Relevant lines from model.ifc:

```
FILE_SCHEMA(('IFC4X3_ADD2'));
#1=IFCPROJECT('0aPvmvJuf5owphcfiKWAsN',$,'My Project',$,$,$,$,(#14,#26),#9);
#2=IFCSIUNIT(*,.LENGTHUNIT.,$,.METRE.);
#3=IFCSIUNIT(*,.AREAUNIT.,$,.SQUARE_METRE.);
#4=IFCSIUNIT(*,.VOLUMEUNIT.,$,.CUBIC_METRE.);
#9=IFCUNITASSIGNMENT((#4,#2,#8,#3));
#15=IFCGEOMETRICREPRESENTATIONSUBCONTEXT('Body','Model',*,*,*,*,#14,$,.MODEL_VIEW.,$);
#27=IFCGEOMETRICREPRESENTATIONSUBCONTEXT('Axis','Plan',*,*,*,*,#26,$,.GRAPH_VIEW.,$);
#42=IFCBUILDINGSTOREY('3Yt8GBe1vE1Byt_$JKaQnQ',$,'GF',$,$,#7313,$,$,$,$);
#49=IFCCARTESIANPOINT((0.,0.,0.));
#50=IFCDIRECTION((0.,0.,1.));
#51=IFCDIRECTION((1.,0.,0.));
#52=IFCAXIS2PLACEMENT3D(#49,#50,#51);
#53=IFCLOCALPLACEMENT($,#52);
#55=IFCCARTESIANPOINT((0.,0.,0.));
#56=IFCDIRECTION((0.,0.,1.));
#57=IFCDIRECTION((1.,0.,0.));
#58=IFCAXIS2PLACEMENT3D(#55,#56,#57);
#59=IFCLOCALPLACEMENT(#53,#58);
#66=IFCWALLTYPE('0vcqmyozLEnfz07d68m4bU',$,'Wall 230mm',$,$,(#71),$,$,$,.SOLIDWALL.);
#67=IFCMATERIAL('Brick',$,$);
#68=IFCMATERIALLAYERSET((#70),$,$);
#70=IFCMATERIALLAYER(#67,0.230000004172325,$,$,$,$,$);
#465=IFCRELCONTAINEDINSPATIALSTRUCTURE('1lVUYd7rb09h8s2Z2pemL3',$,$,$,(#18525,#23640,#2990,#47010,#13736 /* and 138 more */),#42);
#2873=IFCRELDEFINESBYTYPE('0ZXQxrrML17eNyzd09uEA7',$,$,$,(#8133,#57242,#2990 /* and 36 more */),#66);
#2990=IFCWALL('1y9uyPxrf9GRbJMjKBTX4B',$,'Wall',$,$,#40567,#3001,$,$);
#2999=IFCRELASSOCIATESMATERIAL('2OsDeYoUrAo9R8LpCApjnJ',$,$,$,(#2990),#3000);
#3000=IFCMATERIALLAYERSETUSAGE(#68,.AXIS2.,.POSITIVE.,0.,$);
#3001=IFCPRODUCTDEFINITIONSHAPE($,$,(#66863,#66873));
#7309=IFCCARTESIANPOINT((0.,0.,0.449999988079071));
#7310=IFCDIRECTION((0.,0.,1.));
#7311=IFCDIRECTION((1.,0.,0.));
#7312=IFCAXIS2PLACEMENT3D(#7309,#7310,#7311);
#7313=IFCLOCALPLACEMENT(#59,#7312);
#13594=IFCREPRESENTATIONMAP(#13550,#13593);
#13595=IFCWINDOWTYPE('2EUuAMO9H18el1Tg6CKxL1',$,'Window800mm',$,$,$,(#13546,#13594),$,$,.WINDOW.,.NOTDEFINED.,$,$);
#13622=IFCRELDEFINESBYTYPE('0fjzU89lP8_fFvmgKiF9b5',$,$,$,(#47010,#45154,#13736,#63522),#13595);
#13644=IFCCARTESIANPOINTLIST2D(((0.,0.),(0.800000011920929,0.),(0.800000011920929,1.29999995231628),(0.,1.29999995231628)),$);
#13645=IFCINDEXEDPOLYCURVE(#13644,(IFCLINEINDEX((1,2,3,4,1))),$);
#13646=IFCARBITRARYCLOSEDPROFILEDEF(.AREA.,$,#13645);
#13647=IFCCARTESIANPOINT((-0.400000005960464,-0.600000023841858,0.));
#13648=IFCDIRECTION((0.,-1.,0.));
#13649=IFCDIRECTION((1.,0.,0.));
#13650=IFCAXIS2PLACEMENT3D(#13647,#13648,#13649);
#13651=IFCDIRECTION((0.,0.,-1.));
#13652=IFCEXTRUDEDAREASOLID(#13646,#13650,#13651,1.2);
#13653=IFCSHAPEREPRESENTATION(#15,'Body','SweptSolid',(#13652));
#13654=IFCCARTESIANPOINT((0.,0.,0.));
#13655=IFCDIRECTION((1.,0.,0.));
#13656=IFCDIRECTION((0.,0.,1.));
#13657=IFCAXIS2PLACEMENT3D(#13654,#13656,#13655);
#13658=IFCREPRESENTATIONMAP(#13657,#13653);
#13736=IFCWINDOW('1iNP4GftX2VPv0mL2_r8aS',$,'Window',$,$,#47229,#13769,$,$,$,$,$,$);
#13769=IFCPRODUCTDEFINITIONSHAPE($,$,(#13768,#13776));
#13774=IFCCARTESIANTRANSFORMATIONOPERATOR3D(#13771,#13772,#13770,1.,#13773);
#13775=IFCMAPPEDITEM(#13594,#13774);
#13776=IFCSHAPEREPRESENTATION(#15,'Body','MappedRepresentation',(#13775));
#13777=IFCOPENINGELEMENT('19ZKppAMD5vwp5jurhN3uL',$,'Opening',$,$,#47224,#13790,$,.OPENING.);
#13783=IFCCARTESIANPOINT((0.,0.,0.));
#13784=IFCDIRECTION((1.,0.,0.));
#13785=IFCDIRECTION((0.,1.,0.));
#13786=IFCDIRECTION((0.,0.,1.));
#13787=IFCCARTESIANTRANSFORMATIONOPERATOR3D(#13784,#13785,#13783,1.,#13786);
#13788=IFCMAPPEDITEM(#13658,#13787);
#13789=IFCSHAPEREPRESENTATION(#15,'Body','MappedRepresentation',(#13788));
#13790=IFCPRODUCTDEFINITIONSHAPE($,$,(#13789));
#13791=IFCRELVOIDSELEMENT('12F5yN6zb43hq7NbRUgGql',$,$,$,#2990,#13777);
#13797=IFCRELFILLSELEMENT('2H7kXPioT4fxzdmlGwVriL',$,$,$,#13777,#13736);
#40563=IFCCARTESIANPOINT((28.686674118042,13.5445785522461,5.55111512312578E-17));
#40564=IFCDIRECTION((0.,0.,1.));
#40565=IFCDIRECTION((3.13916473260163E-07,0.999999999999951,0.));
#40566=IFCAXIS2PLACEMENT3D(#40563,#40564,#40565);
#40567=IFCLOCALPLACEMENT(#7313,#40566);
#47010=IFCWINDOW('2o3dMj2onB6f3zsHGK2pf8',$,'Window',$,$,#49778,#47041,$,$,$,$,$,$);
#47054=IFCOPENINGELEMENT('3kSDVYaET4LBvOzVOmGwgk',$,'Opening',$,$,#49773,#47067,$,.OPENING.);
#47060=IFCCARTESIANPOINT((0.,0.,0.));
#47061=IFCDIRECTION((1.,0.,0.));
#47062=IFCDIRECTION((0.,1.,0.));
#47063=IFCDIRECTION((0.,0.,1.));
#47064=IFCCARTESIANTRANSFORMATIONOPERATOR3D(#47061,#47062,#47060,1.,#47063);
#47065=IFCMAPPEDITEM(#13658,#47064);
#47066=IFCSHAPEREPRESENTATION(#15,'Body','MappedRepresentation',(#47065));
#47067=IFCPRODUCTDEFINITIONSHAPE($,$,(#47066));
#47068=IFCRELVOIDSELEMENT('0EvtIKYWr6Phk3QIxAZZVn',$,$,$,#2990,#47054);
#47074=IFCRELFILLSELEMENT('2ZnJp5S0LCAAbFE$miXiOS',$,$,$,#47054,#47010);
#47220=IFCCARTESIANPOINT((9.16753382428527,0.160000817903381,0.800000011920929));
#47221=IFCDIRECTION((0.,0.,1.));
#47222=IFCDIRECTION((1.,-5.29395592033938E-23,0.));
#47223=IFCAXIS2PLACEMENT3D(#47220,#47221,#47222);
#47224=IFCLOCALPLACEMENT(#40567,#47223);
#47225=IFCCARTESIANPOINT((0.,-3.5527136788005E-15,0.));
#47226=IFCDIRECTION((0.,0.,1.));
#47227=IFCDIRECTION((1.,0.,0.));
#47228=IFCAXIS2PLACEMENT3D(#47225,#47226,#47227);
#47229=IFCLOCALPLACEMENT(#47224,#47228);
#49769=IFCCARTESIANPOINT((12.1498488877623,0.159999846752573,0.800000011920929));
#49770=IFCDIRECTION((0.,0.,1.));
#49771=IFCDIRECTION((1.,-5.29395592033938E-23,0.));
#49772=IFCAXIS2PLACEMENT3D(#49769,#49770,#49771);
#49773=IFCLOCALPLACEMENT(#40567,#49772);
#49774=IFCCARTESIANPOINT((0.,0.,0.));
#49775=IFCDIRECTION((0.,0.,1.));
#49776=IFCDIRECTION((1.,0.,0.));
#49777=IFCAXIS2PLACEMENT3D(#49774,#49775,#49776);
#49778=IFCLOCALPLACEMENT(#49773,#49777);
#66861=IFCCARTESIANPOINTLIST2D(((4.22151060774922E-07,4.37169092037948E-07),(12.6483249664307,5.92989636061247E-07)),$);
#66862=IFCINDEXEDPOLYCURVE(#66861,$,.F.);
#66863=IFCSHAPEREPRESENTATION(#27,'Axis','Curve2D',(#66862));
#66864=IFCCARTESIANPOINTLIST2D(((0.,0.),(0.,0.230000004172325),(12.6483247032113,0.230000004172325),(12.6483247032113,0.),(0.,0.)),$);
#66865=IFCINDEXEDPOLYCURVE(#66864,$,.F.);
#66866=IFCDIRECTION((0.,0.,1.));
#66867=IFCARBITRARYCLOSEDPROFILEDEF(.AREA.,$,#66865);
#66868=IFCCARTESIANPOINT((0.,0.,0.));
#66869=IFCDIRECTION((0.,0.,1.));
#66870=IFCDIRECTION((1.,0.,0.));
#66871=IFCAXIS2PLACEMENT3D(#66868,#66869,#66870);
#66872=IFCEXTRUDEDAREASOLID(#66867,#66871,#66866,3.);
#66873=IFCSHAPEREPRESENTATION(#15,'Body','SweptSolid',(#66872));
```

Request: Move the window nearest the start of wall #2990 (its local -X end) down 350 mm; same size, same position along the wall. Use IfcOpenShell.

```python
import numpy as np
import ifcopenshell
import ifcopenshell.api.geometry
import ifcopenshell.util.placement
import ifcopenshell.util.unit

model = ifcopenshell.open("model.ifc")
unit_scale = ifcopenshell.util.unit.calculate_unit_scale(model)

window = model.by_guid("1iNP4GftX2VPv0mL2_r8aS")
opening = window.FillsVoids[0].RelatingOpeningElement
dz = -0.35

shift = np.array([0.0, 0.0, dz])
# The window is placed relative to its opening, so it follows when the opening moves.
matrix = ifcopenshell.util.placement.get_local_placement(opening.ObjectPlacement)
matrix[:3, 3] += shift
ifcopenshell.api.geometry.edit_object_placement(
    model, product=opening, matrix=matrix, is_si=False, should_transform_children=True
)

print(f"moved by {dz * unit_scale:+.3f} m")

model.write("model_rev.ifc")
```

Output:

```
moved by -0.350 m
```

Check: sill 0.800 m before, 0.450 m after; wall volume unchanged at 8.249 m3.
